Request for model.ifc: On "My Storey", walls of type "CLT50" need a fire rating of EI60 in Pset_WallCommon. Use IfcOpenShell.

First a look at what the model holds.

```python
import ifcopenshell
import ifcopenshell.util.element

model = ifcopenshell.open("model.ifc")
print(model.schema)
storey = next(s for s in model.by_type("IfcBuildingStorey") if s.Name == "My Storey")
walls = [e for e in ifcopenshell.util.element.get_decomposition(storey) if e.is_a("IfcWall")]
seen = {}
for e in walls:
    element_type = ifcopenshell.util.element.get_type(e)
    key = (element_type.Name if element_type != e and element_type else None, ifcopenshell.util.element.get_pset(e, "Pset_WallCommon", "FireRating"))
    seen[key] = seen.get(key, 0) + 1
for (name, value), count in sorted(seen.items(), key=str):
    print(count, "x", name, "|", value)
```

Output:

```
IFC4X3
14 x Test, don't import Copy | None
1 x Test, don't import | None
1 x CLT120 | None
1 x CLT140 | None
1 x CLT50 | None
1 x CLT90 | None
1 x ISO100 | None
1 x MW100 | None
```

```python
import ifcopenshell
import ifcopenshell.api.pset
import ifcopenshell.util.element

model = ifcopenshell.open("model.ifc")

storey = next(s for s in model.by_type("IfcBuildingStorey") if s.Name == "My Storey")
walls = [e for e in ifcopenshell.util.element.get_decomposition(storey) if e.is_a("IfcWall")]

count = 0
for e in walls:
    element_type = ifcopenshell.util.element.get_type(e)
    if element_type in (None, e) or element_type.Name != "CLT50":
        continue
    # add_pset returns the element's existing set when there is one.
    pset = ifcopenshell.api.pset.add_pset(model, product=e, name="Pset_WallCommon")
    ifcopenshell.api.pset.edit_pset(model, pset=pset, properties={"FireRating": "EI60"})
    count += 1

print(count, "walls updated")

model.write("model_rev.ifc")
```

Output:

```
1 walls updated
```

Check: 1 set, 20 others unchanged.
